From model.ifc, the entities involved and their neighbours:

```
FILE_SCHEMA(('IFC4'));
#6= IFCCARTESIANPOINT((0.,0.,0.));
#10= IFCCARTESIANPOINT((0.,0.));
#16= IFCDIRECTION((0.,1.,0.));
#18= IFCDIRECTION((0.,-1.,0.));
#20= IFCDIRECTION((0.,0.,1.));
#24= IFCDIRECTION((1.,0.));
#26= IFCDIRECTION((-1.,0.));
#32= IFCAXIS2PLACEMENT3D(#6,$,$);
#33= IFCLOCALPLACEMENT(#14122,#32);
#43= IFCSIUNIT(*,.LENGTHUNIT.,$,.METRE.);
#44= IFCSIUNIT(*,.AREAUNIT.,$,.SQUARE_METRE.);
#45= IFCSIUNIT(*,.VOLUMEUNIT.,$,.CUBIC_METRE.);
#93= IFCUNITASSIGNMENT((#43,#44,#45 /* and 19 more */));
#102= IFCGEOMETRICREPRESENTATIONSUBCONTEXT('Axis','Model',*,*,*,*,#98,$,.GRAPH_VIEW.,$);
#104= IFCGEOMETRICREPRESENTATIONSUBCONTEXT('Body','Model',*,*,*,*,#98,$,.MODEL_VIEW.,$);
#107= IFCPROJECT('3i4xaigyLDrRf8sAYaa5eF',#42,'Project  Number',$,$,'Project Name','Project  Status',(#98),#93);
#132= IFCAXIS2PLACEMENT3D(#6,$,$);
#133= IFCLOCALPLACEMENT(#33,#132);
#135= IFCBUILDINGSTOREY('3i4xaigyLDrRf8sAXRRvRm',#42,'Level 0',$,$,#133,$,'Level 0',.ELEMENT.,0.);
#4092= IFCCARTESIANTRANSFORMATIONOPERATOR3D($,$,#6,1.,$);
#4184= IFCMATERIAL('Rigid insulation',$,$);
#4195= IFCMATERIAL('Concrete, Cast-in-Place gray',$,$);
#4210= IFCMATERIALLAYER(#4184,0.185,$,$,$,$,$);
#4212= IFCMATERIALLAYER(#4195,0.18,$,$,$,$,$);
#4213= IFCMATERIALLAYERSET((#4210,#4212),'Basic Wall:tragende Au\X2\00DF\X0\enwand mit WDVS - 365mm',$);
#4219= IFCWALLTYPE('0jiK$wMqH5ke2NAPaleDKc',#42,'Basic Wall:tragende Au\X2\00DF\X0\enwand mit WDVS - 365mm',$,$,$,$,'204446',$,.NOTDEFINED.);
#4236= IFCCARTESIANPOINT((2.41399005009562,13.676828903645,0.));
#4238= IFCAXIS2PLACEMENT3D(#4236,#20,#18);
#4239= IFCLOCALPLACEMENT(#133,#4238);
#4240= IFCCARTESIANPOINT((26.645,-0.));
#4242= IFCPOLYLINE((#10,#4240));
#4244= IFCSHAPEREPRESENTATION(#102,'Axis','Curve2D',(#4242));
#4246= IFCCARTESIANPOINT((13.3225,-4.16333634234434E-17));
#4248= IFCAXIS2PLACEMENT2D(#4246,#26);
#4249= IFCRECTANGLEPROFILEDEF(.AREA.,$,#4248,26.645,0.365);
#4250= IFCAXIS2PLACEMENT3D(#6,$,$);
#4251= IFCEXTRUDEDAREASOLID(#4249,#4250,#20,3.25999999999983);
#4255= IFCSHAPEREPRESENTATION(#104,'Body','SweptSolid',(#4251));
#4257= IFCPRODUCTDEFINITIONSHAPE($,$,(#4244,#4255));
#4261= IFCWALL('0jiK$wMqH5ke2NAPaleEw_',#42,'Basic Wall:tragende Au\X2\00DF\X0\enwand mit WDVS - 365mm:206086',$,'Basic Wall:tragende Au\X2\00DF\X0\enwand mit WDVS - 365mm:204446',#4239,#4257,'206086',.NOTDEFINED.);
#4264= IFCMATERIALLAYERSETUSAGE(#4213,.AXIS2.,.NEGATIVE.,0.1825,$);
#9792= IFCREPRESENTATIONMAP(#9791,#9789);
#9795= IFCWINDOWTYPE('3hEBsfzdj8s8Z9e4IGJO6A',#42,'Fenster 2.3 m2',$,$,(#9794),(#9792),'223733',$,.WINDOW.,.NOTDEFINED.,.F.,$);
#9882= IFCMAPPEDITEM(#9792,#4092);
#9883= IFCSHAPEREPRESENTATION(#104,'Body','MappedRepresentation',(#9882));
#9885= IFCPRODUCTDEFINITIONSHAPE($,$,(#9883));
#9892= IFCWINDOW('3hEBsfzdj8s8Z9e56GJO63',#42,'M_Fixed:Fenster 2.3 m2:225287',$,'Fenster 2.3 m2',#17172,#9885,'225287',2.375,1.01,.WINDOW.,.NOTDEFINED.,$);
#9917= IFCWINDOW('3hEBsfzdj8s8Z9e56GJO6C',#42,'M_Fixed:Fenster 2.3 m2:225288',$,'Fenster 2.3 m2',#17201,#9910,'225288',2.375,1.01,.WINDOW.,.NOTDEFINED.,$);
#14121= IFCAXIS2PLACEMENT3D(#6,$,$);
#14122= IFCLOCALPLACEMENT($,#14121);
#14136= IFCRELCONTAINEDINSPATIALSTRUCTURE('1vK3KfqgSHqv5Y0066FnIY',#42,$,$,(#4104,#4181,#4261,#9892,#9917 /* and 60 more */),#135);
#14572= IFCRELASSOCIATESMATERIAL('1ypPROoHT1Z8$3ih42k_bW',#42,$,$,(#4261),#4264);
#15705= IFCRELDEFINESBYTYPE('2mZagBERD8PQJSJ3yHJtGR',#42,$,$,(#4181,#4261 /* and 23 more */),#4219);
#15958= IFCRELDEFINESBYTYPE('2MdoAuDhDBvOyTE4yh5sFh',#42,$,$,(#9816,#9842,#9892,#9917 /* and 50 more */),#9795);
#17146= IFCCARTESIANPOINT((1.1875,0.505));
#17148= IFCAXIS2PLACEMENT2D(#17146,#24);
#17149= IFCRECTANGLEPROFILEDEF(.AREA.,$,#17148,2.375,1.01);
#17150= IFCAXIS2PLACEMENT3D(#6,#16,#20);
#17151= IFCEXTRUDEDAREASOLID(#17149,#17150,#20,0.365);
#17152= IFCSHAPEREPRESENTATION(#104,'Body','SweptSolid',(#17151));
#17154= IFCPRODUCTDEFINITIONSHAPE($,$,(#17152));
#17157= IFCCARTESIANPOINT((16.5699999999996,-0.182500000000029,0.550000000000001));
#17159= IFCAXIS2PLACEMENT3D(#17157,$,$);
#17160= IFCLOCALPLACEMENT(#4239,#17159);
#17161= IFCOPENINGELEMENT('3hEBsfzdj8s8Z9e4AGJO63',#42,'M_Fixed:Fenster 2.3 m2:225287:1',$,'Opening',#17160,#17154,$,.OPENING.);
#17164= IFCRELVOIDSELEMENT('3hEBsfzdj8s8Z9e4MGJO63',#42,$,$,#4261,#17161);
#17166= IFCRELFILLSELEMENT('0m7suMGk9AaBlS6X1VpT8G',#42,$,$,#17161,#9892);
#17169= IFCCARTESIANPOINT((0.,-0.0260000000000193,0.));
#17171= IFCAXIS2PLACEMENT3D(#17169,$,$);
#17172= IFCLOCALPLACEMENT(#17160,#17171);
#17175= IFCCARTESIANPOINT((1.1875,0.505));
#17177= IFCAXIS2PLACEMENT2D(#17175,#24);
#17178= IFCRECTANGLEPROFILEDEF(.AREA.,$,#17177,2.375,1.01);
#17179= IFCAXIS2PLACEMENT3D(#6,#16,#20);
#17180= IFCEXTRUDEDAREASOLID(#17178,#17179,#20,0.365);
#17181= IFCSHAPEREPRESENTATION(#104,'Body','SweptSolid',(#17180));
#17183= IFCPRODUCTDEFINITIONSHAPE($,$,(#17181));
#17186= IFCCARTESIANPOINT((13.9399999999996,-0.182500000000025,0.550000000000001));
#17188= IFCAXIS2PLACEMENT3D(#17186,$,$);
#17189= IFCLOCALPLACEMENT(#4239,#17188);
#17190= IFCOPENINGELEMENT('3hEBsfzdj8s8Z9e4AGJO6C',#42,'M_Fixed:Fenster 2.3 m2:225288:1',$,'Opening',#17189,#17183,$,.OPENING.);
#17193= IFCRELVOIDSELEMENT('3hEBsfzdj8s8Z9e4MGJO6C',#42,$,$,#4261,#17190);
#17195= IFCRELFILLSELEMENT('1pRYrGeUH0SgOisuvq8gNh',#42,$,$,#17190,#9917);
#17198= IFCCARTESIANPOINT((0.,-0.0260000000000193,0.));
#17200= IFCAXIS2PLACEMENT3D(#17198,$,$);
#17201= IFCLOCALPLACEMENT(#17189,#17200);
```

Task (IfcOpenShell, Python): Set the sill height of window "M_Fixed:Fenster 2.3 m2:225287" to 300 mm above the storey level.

```python
import numpy as np
import ifcopenshell
import ifcopenshell.api.geometry
import ifcopenshell.geom
import ifcopenshell.util.element
import ifcopenshell.util.placement
import ifcopenshell.util.shape
import ifcopenshell.util.unit

model = ifcopenshell.open("model.ifc")
unit_scale = ifcopenshell.util.unit.calculate_unit_scale(model)

window = model.by_guid("3hEBsfzdj8s8Z9e56GJO63")
opening = window.FillsVoids[0].RelatingOpeningElement
storey = ifcopenshell.util.element.get_container(window, ifc_class="IfcBuildingStorey")
level = ifcopenshell.util.placement.get_local_placement(storey.ObjectPlacement)[2, 3]

# The opening's origin need not be at the sill, so measure its lowest point.
shape = ifcopenshell.geom.create_shape(ifcopenshell.geom.settings(), opening)
bottom = ifcopenshell.util.shape.get_shape_bottom_elevation(shape, shape.geometry) / unit_scale
dz = level + 0.3 - bottom

shift = np.array([0.0, 0.0, dz])
# The window is placed relative to its opening, so it follows when the opening moves.
matrix = ifcopenshell.util.placement.get_local_placement(opening.ObjectPlacement)
matrix[:3, 3] += shift
ifcopenshell.api.geometry.edit_object_placement(
    model, product=opening, matrix=matrix, is_si=False, should_transform_children=True
)

print(f"moved by {dz * unit_scale:+.3f} m")

model.write("model_edited.ifc")
```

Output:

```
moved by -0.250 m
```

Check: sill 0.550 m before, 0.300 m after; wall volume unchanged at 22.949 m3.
